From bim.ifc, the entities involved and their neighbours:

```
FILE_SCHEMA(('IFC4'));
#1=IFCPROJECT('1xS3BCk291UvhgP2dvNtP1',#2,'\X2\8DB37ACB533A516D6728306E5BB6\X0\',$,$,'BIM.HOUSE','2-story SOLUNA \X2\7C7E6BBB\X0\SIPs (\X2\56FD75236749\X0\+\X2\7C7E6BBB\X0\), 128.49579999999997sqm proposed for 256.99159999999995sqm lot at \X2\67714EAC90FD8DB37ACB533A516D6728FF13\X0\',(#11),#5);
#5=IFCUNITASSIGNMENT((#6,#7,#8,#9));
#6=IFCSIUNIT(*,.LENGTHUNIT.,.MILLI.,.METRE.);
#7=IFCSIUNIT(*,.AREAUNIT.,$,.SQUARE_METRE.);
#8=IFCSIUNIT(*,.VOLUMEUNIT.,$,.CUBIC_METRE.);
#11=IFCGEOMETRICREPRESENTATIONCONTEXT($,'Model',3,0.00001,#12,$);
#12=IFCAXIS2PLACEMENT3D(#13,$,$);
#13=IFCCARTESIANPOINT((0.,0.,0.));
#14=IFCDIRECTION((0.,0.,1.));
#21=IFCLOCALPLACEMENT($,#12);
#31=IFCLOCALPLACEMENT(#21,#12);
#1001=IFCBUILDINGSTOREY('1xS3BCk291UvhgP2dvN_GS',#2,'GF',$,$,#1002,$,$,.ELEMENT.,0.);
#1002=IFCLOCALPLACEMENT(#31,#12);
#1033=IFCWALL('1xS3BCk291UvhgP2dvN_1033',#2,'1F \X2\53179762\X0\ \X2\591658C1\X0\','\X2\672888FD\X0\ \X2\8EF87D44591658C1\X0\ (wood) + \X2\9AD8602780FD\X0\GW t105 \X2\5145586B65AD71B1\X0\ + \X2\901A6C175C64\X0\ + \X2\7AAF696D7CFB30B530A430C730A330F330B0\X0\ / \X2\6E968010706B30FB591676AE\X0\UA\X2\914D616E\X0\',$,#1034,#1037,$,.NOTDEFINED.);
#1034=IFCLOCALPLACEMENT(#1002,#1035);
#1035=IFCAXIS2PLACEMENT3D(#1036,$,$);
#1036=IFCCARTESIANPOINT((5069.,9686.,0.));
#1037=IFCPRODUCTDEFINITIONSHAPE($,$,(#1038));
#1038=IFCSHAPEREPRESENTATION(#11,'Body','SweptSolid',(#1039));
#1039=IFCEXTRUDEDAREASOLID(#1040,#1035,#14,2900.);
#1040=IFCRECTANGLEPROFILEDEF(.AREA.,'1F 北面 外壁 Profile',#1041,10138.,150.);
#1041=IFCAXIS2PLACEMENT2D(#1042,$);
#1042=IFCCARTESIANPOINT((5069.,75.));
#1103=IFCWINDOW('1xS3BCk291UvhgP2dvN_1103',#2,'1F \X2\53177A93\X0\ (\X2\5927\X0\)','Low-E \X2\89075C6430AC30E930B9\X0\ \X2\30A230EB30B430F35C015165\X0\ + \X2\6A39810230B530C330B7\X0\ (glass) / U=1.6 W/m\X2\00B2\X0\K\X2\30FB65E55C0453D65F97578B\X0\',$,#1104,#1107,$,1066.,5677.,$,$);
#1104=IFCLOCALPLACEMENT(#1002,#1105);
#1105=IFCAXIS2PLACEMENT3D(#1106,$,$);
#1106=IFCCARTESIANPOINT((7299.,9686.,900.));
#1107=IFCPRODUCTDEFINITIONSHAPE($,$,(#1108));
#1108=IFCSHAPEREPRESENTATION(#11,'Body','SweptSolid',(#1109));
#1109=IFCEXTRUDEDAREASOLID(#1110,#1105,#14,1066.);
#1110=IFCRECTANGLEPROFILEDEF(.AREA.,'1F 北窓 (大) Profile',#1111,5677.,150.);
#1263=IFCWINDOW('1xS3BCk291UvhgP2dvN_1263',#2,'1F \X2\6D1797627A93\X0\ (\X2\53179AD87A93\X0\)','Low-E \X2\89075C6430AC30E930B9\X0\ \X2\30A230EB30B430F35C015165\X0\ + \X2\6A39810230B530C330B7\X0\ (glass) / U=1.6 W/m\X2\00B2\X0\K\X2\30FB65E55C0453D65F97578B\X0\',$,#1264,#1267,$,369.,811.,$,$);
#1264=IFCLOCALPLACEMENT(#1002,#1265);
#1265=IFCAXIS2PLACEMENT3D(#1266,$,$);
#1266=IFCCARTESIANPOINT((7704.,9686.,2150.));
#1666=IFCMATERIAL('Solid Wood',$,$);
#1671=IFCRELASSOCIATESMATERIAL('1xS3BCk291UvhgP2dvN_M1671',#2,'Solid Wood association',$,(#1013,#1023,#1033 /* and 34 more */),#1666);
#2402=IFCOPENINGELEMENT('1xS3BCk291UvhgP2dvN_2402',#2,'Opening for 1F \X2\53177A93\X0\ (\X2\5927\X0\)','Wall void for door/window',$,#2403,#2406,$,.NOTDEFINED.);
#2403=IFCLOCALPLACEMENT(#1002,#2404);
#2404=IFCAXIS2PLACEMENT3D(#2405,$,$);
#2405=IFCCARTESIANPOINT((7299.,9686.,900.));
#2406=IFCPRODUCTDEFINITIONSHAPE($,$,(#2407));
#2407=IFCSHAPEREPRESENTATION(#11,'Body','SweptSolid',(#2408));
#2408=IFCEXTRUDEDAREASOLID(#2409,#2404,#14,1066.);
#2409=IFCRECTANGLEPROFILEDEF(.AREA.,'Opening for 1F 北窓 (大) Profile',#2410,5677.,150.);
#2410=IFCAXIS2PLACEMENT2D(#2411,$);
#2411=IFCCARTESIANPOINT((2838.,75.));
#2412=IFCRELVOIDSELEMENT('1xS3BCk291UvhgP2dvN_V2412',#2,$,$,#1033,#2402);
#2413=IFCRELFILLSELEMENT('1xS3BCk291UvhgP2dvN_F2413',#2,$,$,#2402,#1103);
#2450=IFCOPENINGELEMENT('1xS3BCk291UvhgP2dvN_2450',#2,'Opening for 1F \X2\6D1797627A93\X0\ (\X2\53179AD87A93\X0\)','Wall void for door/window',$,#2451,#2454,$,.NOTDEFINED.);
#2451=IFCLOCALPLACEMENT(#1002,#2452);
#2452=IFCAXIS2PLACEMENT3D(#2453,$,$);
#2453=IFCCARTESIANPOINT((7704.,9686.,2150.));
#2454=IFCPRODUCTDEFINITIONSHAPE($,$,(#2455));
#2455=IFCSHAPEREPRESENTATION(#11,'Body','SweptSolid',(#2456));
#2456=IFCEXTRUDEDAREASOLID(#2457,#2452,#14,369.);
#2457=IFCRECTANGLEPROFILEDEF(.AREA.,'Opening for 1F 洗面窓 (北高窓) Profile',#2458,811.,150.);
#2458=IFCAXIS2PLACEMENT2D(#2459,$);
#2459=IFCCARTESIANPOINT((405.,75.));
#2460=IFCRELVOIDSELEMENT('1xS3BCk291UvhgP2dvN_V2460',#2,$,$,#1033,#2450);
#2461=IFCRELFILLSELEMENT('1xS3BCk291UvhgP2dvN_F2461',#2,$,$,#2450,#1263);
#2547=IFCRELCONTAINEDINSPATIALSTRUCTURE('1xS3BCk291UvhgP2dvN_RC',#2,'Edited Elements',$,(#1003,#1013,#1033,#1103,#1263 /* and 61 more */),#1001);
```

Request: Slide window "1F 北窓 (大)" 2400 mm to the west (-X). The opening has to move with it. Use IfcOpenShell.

```python
import ifcopenshell
import ifcopenshell.api.geometry
import ifcopenshell.util.placement
import ifcopenshell.util.unit

model = ifcopenshell.open("bim.ifc")
unit_scale = ifcopenshell.util.unit.calculate_unit_scale(model)

window = model.by_id(1103)
opening = window.FillsVoids[0].RelatingOpeningElement
wall = opening.VoidsElements[0].RelatingBuildingElement

wall_matrix = ifcopenshell.util.placement.get_local_placement(wall.ObjectPlacement)
shift = wall_matrix[:3, 0] * -2.4 / unit_scale
before = ifcopenshell.util.placement.get_local_placement(window.ObjectPlacement)[:3, 3].copy()

# The window is not placed relative to its opening, so move both.
for product in (opening, window):
    matrix = ifcopenshell.util.placement.get_local_placement(product.ObjectPlacement)
    matrix[:3, 3] += shift
    ifcopenshell.api.geometry.edit_object_placement(model, product=product, matrix=matrix, is_si=False)

after = ifcopenshell.util.placement.get_local_placement(window.ObjectPlacement)[:3, 3]
print("window moved by", (after - before).round(3) + 0.0)

model.write("bim_v2.ifc")
```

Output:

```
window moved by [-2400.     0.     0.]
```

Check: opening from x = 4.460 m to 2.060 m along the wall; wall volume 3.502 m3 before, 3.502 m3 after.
